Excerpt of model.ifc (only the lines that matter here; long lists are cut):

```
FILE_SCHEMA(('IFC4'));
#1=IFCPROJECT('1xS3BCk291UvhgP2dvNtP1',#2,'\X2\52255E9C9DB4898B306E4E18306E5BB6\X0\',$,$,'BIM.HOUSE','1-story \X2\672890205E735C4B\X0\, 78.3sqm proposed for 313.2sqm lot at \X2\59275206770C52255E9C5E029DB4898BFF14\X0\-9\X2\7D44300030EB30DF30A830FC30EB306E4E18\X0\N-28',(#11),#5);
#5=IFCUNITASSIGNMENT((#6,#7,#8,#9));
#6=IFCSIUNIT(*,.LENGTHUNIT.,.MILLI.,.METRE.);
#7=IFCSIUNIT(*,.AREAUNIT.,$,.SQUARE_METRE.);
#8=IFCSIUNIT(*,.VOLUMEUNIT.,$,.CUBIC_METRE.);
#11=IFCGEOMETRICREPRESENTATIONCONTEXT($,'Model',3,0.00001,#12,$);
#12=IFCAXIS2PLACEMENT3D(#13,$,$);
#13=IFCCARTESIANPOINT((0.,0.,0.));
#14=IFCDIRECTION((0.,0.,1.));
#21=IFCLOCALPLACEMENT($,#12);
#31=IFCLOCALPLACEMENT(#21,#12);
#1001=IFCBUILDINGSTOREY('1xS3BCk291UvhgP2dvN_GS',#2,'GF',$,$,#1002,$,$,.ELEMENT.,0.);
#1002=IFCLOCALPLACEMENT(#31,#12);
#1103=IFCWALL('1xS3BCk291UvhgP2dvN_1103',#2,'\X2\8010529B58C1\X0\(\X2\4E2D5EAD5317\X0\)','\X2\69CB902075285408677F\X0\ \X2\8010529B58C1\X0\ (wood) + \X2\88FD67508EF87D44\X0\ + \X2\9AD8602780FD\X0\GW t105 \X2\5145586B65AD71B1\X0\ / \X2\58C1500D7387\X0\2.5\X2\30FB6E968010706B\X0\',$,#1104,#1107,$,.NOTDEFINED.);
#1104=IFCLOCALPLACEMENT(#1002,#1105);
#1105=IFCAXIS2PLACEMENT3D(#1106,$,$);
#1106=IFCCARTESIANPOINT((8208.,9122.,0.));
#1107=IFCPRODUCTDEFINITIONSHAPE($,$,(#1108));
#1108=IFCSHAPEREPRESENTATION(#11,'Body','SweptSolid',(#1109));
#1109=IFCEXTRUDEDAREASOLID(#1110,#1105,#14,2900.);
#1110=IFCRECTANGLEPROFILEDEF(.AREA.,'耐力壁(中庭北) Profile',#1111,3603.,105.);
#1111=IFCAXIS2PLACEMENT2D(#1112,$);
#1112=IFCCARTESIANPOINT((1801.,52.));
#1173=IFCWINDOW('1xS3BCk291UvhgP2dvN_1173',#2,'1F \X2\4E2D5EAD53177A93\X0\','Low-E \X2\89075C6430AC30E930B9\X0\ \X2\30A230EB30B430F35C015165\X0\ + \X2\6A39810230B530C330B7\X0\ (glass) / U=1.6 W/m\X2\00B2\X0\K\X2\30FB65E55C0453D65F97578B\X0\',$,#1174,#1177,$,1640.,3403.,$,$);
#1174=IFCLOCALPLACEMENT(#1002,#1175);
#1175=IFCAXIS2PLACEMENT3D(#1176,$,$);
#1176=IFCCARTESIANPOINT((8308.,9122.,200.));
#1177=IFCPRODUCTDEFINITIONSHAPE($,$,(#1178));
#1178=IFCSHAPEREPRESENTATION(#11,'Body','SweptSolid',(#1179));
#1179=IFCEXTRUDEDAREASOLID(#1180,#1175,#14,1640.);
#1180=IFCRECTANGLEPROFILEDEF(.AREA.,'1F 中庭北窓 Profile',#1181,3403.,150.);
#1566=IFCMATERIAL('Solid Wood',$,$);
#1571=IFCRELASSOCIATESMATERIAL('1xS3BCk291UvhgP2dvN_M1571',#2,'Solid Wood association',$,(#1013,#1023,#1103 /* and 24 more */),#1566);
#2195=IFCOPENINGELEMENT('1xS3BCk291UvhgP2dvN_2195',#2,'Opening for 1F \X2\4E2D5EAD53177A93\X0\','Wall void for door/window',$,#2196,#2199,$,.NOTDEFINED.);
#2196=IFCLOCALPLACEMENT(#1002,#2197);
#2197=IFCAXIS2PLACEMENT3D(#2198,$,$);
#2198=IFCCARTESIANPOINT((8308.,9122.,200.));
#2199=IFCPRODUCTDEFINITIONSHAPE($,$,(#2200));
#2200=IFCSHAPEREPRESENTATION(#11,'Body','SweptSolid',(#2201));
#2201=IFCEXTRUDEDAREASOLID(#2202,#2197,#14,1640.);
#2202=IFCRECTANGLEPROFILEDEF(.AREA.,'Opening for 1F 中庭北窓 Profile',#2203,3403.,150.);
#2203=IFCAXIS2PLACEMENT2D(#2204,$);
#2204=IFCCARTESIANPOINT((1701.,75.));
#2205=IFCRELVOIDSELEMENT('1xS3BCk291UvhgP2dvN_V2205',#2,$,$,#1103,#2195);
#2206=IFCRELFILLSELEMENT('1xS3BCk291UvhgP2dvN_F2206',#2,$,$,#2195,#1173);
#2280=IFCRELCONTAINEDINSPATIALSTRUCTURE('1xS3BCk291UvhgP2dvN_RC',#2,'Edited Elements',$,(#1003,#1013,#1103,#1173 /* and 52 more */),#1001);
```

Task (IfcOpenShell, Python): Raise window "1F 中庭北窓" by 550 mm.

```python
import numpy as np
import ifcopenshell
import ifcopenshell.api.geometry
import ifcopenshell.util.placement
import ifcopenshell.util.unit

model = ifcopenshell.open("model.ifc")
unit_scale = ifcopenshell.util.unit.calculate_unit_scale(model)

window = model.by_guid("1xS3BCk291UvhgP2dvN_1173")
opening = window.FillsVoids[0].RelatingOpeningElement
dz = 550.0

shift = np.array([0.0, 0.0, dz])
# The window is not placed relative to its opening, so move both.
for product in (opening, window):
    matrix = ifcopenshell.util.placement.get_local_placement(product.ObjectPlacement)
    matrix[:3, 3] += shift
    ifcopenshell.api.geometry.edit_object_placement(model, product=product, matrix=matrix, is_si=False)

print(f"moved by {dz * unit_scale:+.3f} m")

model.write("model_v2.ifc")
```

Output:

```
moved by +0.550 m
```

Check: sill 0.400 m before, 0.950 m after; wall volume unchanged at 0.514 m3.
